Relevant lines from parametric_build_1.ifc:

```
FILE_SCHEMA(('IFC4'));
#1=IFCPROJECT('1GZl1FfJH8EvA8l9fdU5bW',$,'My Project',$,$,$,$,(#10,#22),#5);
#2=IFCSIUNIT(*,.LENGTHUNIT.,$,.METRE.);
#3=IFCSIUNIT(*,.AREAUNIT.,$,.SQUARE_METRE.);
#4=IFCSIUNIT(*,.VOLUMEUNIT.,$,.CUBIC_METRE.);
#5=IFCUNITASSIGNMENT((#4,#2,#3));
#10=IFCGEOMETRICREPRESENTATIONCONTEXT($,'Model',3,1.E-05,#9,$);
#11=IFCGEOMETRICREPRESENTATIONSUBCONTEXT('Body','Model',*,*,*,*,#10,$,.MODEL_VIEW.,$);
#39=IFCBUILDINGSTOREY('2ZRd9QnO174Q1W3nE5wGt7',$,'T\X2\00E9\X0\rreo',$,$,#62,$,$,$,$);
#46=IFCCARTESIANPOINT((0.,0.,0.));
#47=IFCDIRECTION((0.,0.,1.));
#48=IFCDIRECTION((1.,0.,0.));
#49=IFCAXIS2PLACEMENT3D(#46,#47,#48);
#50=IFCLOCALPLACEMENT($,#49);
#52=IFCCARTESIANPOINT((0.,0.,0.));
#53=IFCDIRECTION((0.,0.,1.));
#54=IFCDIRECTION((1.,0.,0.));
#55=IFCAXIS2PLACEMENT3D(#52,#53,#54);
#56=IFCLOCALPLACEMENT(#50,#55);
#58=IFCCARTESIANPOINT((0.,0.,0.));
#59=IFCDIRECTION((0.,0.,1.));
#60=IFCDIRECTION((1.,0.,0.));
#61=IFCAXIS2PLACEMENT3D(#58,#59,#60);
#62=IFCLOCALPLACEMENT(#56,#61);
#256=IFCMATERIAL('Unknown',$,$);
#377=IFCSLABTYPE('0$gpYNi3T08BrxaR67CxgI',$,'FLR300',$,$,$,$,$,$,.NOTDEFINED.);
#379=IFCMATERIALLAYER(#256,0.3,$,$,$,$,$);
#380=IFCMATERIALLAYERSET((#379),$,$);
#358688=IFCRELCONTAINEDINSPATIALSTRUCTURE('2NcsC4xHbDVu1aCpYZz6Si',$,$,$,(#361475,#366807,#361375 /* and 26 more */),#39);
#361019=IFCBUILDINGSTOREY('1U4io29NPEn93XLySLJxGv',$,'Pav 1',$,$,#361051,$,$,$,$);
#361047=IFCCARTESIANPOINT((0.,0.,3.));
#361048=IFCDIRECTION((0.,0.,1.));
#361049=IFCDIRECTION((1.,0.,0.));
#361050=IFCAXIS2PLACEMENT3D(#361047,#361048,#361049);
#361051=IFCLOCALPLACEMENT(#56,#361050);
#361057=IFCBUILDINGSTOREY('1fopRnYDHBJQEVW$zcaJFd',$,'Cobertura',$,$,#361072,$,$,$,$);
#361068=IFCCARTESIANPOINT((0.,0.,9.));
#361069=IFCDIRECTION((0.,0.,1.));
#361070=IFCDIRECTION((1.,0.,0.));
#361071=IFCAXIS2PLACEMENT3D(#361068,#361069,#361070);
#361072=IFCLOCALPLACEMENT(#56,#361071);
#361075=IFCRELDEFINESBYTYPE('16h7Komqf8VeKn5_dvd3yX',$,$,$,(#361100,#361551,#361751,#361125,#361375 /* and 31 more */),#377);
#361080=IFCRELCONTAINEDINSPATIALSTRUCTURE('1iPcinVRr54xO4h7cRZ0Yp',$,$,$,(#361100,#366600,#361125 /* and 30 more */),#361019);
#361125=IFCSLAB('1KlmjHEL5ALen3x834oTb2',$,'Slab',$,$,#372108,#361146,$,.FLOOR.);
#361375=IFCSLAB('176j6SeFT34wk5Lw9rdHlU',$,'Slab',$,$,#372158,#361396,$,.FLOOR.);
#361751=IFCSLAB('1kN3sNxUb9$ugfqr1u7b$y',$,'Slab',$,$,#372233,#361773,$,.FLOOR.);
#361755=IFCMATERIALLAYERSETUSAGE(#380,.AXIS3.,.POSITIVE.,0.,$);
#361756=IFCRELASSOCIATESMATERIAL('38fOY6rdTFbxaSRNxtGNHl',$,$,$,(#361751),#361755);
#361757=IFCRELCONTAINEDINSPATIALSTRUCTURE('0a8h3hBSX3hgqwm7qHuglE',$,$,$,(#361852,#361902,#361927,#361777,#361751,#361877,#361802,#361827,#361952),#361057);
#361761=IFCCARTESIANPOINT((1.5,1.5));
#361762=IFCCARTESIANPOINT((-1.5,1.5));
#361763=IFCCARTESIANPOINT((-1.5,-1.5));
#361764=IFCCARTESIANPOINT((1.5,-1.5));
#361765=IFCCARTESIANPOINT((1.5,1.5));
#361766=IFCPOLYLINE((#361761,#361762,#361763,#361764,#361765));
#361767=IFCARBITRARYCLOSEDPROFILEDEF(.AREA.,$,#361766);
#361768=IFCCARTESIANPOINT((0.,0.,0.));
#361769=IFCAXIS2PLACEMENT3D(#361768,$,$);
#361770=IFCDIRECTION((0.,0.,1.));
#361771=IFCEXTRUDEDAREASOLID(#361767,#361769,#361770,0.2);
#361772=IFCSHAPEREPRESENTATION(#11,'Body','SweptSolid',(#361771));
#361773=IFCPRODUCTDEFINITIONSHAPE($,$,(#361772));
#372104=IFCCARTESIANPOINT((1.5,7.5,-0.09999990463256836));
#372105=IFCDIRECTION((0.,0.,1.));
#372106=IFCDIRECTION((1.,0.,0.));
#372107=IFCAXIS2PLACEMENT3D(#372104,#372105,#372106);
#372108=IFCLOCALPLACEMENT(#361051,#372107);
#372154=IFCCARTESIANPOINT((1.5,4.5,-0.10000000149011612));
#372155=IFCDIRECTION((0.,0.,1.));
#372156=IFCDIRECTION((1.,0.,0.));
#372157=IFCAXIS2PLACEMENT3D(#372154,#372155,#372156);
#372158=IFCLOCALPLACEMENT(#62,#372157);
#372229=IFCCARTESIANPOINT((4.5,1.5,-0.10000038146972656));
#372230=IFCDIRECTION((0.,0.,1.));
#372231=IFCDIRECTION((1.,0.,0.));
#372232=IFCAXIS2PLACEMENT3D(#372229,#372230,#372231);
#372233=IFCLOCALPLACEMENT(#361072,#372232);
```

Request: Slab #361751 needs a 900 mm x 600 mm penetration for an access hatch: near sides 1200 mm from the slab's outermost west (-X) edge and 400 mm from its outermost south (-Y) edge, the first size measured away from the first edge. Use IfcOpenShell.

```python
import numpy as np
import ifcopenshell
import ifcopenshell.api.feature
import ifcopenshell.api.geometry
import ifcopenshell.api.root
import ifcopenshell.geom
import ifcopenshell.util.placement
import ifcopenshell.util.representation
import ifcopenshell.util.shape
import ifcopenshell.util.unit

model = ifcopenshell.open("parametric_build_1.ifc")
unit_scale = ifcopenshell.util.unit.calculate_unit_scale(model)
settings = ifcopenshell.geom.settings()


def volume(element):
    """Net volume in cubic metres, openings subtracted."""
    shape = ifcopenshell.geom.create_shape(settings, element)
    return ifcopenshell.util.shape.get_volume(shape.geometry)


slab = model.by_guid("1kN3sNxUb9$ugfqr1u7b$y")
before = volume(slab)

# Extent in the slab's own axes, in metres. The edges named are its -X and -Y sides.
slab_shape = ifcopenshell.geom.create_shape(settings, slab)
vertices = ifcopenshell.util.shape.get_vertices(slab_shape.geometry)
x_min, y_min, bottom = vertices.min(axis=0)
top = vertices[:, 2].max()

opening = ifcopenshell.api.root.create_entity(model, ifc_class="IfcOpeningElement", name="Access hatch opening", predefined_type="OPENING")
context = ifcopenshell.util.representation.get_context(model, "Model", "Body", "MODEL_VIEW")
width, depth = 0.9, 0.6
outline = [(0.0, 0.0), (width, 0.0), (width, depth), (0.0, depth), (0.0, 0.0)]
# Overshoot both faces by 50 mm so the cut is clean.
shape = ifcopenshell.api.geometry.add_slab_representation(
    model, context=context, depth=top - bottom + 0.1, polyline=outline
)
ifcopenshell.api.geometry.assign_representation(model, product=opening, representation=shape)

matrix = ifcopenshell.util.placement.get_local_placement(slab.ObjectPlacement)
matrix[:, 3] = matrix @ np.append(np.array([x_min + 1.2, y_min + 0.4, bottom - 0.05]) / unit_scale, 1.0)
ifcopenshell.api.geometry.edit_object_placement(model, product=opening, matrix=matrix, is_si=False)
ifcopenshell.api.feature.add_feature(model, feature=opening, element=slab)

after = volume(slab)

print(f"slab volume {before:.3f} -> {after:.3f} m3")

model.write("parametric_build_1_edited.ifc")
```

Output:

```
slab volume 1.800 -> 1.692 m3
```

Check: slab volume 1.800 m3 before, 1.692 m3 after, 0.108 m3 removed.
